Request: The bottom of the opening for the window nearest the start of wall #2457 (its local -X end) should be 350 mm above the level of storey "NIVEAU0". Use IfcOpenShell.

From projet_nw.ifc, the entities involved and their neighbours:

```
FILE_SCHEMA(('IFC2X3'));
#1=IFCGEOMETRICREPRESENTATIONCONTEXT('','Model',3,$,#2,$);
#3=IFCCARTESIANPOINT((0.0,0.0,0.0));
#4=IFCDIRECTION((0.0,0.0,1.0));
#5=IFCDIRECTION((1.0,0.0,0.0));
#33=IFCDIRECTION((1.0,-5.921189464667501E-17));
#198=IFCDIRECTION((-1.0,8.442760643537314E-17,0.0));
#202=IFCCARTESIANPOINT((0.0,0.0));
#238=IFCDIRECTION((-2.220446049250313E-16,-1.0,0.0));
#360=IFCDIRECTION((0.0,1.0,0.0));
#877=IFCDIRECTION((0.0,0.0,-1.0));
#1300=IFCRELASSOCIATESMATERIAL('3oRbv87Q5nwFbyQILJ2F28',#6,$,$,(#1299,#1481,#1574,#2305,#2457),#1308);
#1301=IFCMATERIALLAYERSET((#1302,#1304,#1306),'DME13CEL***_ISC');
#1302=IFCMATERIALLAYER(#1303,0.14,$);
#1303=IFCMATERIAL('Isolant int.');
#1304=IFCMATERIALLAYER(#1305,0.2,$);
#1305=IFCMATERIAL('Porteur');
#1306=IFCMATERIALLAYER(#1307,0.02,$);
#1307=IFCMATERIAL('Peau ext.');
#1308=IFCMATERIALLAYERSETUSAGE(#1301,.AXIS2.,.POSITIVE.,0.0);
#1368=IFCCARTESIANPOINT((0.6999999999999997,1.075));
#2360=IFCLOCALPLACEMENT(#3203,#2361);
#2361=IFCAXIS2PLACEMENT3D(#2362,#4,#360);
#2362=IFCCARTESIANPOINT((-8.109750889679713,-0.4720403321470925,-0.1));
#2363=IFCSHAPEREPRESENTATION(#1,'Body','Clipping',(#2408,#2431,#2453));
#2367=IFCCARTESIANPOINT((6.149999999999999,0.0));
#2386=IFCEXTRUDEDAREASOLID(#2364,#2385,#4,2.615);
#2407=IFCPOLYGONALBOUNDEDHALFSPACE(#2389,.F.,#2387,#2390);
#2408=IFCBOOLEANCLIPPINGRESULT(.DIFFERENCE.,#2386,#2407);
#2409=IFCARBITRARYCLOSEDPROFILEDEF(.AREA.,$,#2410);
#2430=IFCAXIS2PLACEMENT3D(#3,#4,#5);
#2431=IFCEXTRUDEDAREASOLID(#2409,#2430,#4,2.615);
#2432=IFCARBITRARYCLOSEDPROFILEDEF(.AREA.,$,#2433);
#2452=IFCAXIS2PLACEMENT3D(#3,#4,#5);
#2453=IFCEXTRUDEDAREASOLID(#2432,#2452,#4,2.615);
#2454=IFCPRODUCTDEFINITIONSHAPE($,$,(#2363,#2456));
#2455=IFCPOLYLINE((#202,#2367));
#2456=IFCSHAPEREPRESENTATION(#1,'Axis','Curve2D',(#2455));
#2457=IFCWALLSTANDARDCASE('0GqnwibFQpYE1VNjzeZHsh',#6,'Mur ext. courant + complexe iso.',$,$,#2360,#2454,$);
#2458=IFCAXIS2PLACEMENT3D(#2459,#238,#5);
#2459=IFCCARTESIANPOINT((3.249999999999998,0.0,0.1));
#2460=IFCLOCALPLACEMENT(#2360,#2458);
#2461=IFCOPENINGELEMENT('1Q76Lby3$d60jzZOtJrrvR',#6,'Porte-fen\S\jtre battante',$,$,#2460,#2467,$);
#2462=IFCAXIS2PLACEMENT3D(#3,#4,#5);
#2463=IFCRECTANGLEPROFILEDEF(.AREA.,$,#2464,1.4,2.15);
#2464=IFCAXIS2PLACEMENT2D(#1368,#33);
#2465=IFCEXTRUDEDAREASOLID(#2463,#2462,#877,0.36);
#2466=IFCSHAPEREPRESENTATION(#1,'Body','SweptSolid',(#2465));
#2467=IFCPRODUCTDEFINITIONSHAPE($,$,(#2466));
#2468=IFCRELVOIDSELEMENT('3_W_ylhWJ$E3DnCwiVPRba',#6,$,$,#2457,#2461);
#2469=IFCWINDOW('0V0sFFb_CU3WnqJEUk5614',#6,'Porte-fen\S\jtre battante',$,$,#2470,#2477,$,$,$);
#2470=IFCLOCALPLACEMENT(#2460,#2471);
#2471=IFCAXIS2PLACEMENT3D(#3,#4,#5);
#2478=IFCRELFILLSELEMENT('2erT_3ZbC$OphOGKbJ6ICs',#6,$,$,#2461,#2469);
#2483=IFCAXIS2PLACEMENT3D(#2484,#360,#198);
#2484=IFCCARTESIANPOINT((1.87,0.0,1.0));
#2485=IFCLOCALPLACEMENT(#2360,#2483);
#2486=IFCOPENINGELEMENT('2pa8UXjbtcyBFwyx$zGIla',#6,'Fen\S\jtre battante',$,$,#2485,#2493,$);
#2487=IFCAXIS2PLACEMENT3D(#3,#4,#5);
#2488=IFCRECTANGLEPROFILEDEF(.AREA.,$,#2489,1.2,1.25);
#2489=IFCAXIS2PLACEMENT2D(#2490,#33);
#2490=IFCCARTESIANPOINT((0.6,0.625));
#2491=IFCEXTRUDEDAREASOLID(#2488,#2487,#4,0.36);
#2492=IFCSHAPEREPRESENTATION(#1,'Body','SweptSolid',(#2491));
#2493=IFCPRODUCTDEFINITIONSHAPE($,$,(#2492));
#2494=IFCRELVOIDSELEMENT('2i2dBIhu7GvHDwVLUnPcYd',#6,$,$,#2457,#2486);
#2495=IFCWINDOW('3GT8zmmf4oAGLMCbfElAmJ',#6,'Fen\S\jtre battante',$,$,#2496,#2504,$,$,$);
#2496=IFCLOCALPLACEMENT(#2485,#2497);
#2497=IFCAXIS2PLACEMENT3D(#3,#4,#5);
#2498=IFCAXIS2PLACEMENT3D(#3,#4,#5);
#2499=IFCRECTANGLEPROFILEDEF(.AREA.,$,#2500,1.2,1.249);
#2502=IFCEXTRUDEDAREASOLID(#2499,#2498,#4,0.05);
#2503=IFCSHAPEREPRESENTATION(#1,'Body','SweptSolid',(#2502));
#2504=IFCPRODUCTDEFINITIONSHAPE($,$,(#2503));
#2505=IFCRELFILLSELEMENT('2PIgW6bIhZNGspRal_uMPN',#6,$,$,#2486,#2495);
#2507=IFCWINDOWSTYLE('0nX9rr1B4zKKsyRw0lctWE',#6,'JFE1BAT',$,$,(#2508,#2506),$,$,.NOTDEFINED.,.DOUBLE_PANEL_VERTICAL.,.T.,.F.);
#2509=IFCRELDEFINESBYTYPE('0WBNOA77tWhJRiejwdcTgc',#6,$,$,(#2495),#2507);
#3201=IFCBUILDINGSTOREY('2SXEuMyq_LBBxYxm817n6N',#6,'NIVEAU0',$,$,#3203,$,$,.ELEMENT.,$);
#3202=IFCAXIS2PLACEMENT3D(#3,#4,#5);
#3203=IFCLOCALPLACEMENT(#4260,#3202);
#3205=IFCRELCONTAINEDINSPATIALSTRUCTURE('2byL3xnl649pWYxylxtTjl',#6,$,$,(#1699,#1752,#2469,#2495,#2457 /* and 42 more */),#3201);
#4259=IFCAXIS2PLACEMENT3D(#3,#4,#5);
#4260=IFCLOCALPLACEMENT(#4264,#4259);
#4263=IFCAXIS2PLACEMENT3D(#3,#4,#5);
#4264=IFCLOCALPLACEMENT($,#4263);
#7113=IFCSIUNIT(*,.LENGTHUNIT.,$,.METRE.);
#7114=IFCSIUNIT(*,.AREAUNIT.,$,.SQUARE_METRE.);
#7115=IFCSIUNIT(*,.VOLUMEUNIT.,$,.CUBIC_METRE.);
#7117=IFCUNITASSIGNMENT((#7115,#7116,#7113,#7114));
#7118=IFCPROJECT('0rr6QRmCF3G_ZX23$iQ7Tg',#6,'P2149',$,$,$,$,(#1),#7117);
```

```python
import numpy as np
import ifcopenshell
import ifcopenshell.api.geometry
import ifcopenshell.geom
import ifcopenshell.util.element
import ifcopenshell.util.placement
import ifcopenshell.util.shape
import ifcopenshell.util.unit

model = ifcopenshell.open("projet_nw.ifc")
unit_scale = ifcopenshell.util.unit.calculate_unit_scale(model)

window = model.by_guid("3GT8zmmf4oAGLMCbfElAmJ")
opening = window.FillsVoids[0].RelatingOpeningElement
storey = ifcopenshell.util.element.get_container(window, ifc_class="IfcBuildingStorey")
level = ifcopenshell.util.placement.get_local_placement(storey.ObjectPlacement)[2, 3]

# The opening's origin need not be at the sill, so measure its lowest point.
shape = ifcopenshell.geom.create_shape(ifcopenshell.geom.settings(), opening)
bottom = ifcopenshell.util.shape.get_shape_bottom_elevation(shape, shape.geometry) / unit_scale
dz = level + 0.35 - bottom

shift = np.array([0.0, 0.0, dz])
# The window is placed relative to its opening, so it follows when the opening moves.
matrix = ifcopenshell.util.placement.get_local_placement(opening.ObjectPlacement)
matrix[:3, 3] += shift
ifcopenshell.api.geometry.edit_object_placement(
    model, product=opening, matrix=matrix, is_si=False, should_transform_children=True
)

print(f"moved by {dz * unit_scale:+.3f} m")

model.write("projet_nw_rev.ifc")
```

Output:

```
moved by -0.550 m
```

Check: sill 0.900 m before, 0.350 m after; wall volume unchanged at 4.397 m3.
